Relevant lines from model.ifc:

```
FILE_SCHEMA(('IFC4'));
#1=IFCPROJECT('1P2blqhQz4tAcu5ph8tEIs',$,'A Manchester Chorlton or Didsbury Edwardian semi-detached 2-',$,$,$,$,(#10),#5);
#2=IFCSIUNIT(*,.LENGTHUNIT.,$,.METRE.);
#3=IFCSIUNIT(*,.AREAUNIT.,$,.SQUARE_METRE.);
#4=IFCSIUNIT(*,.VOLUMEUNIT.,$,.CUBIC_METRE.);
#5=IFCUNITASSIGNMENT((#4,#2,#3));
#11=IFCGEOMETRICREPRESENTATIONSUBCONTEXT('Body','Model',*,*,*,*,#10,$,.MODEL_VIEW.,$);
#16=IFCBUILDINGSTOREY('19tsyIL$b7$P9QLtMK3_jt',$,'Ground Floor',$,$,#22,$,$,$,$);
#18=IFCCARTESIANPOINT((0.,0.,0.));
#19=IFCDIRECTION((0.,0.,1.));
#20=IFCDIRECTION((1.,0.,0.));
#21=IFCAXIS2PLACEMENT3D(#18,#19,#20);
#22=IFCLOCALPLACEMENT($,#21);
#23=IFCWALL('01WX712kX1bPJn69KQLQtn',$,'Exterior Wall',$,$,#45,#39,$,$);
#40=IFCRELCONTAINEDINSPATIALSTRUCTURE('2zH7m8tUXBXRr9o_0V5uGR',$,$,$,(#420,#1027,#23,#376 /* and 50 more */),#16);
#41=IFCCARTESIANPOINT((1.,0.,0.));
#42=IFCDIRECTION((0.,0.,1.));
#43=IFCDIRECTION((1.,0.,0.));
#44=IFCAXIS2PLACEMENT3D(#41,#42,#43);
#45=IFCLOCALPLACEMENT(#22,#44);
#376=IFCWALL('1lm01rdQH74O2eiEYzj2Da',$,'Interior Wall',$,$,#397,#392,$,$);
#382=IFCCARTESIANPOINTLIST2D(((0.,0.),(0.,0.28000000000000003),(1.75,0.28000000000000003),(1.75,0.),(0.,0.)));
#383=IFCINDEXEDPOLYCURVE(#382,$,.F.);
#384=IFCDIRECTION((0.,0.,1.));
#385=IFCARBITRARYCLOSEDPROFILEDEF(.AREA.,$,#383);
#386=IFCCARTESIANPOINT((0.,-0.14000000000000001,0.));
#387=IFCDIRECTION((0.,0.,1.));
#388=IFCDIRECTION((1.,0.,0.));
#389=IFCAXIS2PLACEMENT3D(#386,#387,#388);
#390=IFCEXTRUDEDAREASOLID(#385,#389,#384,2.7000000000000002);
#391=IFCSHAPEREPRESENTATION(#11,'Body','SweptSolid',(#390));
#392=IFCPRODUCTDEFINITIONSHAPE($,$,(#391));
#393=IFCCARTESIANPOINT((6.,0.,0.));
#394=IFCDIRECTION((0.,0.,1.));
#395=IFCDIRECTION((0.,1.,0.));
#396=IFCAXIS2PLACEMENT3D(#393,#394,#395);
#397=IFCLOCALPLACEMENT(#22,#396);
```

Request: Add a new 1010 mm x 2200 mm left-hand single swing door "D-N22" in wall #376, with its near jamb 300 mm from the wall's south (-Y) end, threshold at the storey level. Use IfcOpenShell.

```python
import numpy as np
import ifcopenshell
import ifcopenshell.api.feature
import ifcopenshell.api.geometry
import ifcopenshell.api.root
import ifcopenshell.api.spatial
import ifcopenshell.geom
import ifcopenshell.util.element
import ifcopenshell.util.placement
import ifcopenshell.util.representation
import ifcopenshell.util.shape
import ifcopenshell.util.unit

model = ifcopenshell.open("model.ifc")
unit_scale = ifcopenshell.util.unit.calculate_unit_scale(model)
settings = ifcopenshell.geom.settings()


def volume(element):
    """Net volume in cubic metres, openings subtracted."""
    shape = ifcopenshell.geom.create_shape(settings, element)
    return ifcopenshell.util.shape.get_volume(shape.geometry)


wall = model.by_guid("1lm01rdQH74O2eiEYzj2Da")
storey = ifcopenshell.util.element.get_container(wall, ifc_class="IfcBuildingStorey")
context = ifcopenshell.util.representation.get_context(model, "Model", "Body", "MODEL_VIEW")
before = volume(wall)

width, height, from_end, sill = 1.01, 2.2, 0.3, 0.0  # metres

# The wall runs along its own X axis, and the end named is its -X end.
wall_shape = ifcopenshell.geom.create_shape(settings, wall)
x, y, z = ifcopenshell.util.shape.get_vertices(wall_shape.geometry).T
start = x.min() + from_end
face, thickness = float(y.min()), float(y.max() - y.min())
wall_matrix = ifcopenshell.util.placement.get_local_placement(wall.ObjectPlacement)
level = ifcopenshell.util.placement.get_local_placement(storey.ObjectPlacement)[2, 3]


def in_wall(x, y):
    """Placement at x, y metres in the wall's axes, at sill height."""
    matrix = wall_matrix.copy()
    matrix[:, 3] = wall_matrix @ np.array([x / unit_scale, y / unit_scale, 0.0, 1.0])
    matrix[2, 3] = level + sill / unit_scale
    return matrix


# Opening: a box that overshoots both wall faces by 50 mm.
opening = ifcopenshell.api.root.create_entity(model, ifc_class="IfcOpeningElement", predefined_type="OPENING")
box = ifcopenshell.api.geometry.add_wall_representation(
    model, context=context, length=width, height=height, thickness=thickness + 0.1
)
ifcopenshell.api.geometry.assign_representation(model, product=opening, representation=box)
ifcopenshell.api.geometry.edit_object_placement(model, product=opening, matrix=in_wall(start, face - 0.05), is_si=False)
ifcopenshell.api.feature.add_feature(model, feature=opening, element=wall)

door = ifcopenshell.api.root.create_entity(model, ifc_class="IfcDoor", name="D-N22", predefined_type="DOOR")
door.OverallWidth, door.OverallHeight = width / unit_scale, height / unit_scale
door.OperationType = "SINGLE_SWING_LEFT"
body = ifcopenshell.api.geometry.add_door_representation(
    model,
    context=context,
    overall_width=door.OverallWidth,
    overall_height=door.OverallHeight,
    operation_type="SINGLE_SWING_LEFT",
    lining_properties={"LiningDepth": thickness / unit_scale, "ThresholdDepth": thickness / unit_scale},
)
ifcopenshell.api.geometry.assign_representation(model, product=door, representation=body)
ifcopenshell.api.spatial.assign_container(model, products=[door], relating_structure=storey)
ifcopenshell.api.feature.add_filling(model, opening=opening, element=door)

# The lining spans the wall, so the door starts at the wall face.
ifcopenshell.api.geometry.edit_object_placement(model, product=door, matrix=in_wall(start, face), is_si=False)

after = volume(wall)

print(f"wall volume {before:.3f} -> {after:.3f} m3")

model.write("model_updated.ifc")
```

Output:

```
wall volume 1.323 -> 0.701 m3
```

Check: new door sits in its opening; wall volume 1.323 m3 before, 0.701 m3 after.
